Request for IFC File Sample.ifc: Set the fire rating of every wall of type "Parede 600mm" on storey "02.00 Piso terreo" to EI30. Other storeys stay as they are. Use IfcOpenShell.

First a look at what the model holds.

```python
import ifcopenshell
import ifcopenshell.util.element

model = ifcopenshell.open("IFC File Sample.ifc")
print(model.schema)
storey = next(s for s in model.by_type("IfcBuildingStorey") if s.Name == "02.00 Piso terreo")
walls = [e for e in ifcopenshell.util.element.get_decomposition(storey) if e.is_a("IfcWall")]
seen = {}
for e in walls:
    element_type = ifcopenshell.util.element.get_type(e)
    key = (element_type.Name if element_type != e and element_type else None, ifcopenshell.util.element.get_pset(e, "Pset_WallCommon", "FireRating"))
    seen[key] = seen.get(key, 0) + 1
for (name, value), count in sorted(seen.items(), key=str):
    print(count, "x", name, "|", value)
```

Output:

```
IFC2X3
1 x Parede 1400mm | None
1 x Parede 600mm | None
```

```python
import ifcopenshell
import ifcopenshell.api.pset
import ifcopenshell.util.element

model = ifcopenshell.open("IFC File Sample.ifc")

storey = next(s for s in model.by_type("IfcBuildingStorey") if s.Name == "02.00 Piso terreo")
walls = [e for e in ifcopenshell.util.element.get_decomposition(storey) if e.is_a("IfcWall")]

count = 0
for e in walls:
    element_type = ifcopenshell.util.element.get_type(e)
    if element_type in (None, e) or element_type.Name != "Parede 600mm":
        continue
    # add_pset returns the element's existing set when there is one.
    pset = ifcopenshell.api.pset.add_pset(model, product=e, name="Pset_WallCommon")
    ifcopenshell.api.pset.edit_pset(model, pset=pset, properties={"FireRating": "EI30"})
    count += 1

print(count, "walls updated")

model.write("IFC File Sample_updated.ifc")
```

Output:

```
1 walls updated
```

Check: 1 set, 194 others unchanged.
